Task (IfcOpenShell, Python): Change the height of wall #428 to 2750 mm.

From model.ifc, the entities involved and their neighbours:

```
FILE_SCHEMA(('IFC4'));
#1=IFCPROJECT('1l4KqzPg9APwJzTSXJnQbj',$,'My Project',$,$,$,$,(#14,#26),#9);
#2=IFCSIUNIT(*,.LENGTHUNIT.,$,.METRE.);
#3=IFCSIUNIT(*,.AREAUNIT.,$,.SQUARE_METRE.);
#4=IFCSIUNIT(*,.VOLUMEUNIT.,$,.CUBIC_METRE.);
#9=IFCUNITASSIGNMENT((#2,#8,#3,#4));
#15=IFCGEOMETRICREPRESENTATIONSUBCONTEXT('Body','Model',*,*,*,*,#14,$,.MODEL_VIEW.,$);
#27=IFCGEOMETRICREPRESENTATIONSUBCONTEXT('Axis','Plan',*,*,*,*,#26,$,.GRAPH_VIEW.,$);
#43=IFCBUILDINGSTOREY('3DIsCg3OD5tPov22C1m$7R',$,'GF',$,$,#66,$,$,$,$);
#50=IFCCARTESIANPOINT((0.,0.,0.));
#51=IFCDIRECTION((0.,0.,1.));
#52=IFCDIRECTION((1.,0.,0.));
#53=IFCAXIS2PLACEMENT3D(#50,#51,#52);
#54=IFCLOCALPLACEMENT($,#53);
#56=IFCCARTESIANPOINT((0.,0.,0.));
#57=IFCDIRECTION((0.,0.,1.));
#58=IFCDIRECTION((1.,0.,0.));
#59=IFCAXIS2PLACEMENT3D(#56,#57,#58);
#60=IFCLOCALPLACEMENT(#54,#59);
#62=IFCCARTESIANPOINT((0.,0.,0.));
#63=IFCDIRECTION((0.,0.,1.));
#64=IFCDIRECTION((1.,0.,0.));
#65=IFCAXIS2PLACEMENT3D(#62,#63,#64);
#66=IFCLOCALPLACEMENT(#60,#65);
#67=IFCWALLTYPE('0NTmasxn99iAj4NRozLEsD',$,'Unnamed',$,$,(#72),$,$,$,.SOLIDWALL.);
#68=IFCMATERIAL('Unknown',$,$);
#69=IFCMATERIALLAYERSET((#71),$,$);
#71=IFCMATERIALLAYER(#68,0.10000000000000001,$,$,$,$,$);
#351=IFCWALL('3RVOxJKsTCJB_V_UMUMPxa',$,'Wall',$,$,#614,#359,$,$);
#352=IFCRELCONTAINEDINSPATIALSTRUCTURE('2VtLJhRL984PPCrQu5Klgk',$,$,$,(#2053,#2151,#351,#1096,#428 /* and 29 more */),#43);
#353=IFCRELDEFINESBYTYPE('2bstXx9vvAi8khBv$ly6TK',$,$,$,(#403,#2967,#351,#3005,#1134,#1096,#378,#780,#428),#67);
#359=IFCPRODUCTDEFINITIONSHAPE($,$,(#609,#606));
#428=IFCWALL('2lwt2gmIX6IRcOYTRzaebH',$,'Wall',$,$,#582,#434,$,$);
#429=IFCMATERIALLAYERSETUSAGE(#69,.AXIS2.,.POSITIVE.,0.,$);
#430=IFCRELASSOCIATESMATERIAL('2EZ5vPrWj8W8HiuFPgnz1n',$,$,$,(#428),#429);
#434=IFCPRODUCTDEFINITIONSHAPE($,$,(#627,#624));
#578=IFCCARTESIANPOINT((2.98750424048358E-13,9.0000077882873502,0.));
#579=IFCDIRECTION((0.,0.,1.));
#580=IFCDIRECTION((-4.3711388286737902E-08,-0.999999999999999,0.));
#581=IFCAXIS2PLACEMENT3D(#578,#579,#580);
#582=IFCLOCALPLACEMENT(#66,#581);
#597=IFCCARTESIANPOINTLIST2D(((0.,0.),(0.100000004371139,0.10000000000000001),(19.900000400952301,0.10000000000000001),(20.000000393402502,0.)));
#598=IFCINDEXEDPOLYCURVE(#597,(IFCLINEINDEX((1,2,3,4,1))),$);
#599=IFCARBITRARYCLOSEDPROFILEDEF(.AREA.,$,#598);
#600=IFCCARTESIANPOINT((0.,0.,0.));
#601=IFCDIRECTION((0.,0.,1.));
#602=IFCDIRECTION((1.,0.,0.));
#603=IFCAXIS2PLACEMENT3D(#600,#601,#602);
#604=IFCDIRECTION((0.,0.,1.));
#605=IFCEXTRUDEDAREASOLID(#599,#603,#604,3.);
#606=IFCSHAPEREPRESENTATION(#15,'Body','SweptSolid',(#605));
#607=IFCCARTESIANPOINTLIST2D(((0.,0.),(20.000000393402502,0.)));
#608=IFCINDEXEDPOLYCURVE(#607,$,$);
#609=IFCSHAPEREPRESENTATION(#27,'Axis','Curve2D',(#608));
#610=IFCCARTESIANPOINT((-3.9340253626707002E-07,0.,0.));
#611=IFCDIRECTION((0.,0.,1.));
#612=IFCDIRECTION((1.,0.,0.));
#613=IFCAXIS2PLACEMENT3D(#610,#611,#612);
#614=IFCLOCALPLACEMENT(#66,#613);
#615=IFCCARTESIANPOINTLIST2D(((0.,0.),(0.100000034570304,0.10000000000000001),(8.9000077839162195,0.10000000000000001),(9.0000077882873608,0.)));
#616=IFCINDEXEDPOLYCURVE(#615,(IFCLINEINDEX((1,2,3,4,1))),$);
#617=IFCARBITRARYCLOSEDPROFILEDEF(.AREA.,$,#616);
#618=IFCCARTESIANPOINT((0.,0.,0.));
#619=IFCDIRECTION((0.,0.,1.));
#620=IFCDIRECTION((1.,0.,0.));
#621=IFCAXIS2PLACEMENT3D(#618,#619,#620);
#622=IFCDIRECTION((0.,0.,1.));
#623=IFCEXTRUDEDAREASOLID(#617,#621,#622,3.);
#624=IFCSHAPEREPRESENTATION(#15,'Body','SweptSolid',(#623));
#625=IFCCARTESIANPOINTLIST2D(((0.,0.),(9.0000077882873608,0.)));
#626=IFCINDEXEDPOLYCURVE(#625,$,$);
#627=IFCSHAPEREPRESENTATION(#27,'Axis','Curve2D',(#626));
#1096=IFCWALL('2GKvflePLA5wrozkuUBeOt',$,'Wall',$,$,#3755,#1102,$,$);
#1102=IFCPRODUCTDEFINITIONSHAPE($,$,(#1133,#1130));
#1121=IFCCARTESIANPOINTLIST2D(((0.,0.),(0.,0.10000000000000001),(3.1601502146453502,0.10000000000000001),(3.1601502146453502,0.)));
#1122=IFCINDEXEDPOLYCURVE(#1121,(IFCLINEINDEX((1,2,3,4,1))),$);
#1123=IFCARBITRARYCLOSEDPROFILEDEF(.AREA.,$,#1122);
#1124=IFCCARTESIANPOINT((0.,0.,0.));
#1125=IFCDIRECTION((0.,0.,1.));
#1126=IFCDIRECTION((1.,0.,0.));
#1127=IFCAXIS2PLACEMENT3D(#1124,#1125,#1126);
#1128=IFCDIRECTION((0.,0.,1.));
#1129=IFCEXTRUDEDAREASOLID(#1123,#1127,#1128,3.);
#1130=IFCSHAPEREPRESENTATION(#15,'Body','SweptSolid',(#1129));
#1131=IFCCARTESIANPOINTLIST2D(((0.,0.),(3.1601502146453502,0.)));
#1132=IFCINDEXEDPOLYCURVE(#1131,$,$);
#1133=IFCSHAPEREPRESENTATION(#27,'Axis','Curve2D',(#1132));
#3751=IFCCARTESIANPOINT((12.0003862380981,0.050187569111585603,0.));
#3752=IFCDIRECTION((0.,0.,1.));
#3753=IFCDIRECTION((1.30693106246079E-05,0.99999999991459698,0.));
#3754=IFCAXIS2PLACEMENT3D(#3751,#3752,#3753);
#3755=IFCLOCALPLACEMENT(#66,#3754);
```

```python
import ifcopenshell
import ifcopenshell.geom
import ifcopenshell.util.representation
import ifcopenshell.util.shape
import ifcopenshell.util.unit

model = ifcopenshell.open("model.ifc")
unit_scale = ifcopenshell.util.unit.calculate_unit_scale(model)
settings = ifcopenshell.geom.settings()


def volume(element):
    """Net volume in cubic metres, openings subtracted."""
    shape = ifcopenshell.geom.create_shape(settings, element)
    return ifcopenshell.util.shape.get_volume(shape.geometry)


wall = model.by_guid("2lwt2gmIX6IRcOYTRzaebH")
before = volume(wall)

body = ifcopenshell.util.representation.get_representation(wall, "Model", "Body")
solid = body.Items[0]
old_height = solid.Depth
solid.Depth = 2.75 / unit_scale
after = volume(wall)

print(f"height {old_height:g} -> {solid.Depth:g}, volume {before:.3f} -> {after:.3f} m3")

model.write("model_updated.ifc")
```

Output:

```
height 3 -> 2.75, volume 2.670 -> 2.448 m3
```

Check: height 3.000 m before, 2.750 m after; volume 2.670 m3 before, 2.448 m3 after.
